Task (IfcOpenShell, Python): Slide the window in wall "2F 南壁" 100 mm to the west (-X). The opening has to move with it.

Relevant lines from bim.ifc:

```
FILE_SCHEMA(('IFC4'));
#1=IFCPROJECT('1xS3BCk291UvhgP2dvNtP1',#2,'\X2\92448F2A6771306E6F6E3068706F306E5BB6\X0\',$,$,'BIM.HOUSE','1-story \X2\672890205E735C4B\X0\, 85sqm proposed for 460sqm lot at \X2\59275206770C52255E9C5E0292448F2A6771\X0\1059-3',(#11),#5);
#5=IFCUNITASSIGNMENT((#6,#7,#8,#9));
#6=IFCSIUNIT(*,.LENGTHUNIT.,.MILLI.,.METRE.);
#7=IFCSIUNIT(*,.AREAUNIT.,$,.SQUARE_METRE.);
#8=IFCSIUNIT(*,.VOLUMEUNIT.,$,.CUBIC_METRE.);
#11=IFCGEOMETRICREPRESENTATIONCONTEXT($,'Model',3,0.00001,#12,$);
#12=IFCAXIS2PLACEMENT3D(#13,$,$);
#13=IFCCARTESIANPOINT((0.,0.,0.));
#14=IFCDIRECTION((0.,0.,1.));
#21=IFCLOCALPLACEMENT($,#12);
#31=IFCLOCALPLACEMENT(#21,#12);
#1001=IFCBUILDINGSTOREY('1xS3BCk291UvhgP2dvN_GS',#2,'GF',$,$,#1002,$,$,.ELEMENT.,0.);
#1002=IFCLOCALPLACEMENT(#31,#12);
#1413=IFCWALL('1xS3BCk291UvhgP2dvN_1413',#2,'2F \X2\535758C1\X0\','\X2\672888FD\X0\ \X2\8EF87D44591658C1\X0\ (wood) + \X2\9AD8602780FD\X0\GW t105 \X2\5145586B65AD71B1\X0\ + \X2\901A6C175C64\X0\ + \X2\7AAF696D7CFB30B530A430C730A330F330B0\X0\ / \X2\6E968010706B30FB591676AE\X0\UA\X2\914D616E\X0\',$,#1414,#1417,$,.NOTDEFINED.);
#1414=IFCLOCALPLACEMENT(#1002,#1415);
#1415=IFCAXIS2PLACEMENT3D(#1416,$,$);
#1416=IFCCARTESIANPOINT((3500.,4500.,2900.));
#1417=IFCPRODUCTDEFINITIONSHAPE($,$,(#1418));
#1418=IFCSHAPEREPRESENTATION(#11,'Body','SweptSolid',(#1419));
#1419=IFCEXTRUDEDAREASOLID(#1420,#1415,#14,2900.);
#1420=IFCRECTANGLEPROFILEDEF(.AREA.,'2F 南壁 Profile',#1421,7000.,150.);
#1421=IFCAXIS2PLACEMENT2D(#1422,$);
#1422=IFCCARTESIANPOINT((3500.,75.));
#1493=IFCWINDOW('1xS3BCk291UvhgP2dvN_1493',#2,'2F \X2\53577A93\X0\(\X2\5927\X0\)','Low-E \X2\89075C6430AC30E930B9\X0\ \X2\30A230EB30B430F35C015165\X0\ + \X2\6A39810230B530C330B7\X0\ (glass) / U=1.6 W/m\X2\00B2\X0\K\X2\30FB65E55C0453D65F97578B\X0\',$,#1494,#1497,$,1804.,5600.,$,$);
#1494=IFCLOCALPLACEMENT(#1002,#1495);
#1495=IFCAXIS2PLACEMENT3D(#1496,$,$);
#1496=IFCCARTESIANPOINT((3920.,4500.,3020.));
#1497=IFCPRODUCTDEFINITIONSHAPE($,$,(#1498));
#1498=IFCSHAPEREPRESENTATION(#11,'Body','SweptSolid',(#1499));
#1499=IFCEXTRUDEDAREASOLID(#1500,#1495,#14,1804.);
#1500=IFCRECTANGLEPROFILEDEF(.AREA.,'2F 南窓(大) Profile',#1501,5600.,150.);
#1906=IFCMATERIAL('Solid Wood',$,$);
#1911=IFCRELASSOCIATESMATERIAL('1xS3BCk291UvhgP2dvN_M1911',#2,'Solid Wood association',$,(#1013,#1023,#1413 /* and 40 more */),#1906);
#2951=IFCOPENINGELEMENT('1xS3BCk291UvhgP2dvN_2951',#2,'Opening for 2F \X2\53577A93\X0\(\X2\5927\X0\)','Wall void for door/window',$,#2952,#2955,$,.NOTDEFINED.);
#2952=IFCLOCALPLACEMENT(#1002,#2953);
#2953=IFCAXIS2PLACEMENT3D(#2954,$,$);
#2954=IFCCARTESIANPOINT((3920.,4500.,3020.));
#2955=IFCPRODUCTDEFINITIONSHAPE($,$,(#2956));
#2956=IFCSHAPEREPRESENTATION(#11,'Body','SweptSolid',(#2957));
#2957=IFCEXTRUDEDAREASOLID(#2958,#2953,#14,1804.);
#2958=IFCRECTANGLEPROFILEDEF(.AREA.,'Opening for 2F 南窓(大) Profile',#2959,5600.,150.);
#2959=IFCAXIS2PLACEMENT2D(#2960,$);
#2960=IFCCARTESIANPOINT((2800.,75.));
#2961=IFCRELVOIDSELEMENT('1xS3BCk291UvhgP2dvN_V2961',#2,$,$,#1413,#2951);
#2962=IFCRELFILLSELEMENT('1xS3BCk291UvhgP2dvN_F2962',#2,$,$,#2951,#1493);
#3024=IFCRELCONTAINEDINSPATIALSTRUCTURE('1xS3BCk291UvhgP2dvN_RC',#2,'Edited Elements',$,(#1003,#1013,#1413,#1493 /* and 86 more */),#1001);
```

```python
import ifcopenshell
import ifcopenshell.api.geometry
import ifcopenshell.util.placement

model = ifcopenshell.open("bim.ifc")

window = model.by_guid("1xS3BCk291UvhgP2dvN_1493")
opening = window.FillsVoids[0].RelatingOpeningElement
wall = opening.VoidsElements[0].RelatingBuildingElement

wall_matrix = ifcopenshell.util.placement.get_local_placement(wall.ObjectPlacement)
shift = wall_matrix[:3, 0] * -100.0
before = ifcopenshell.util.placement.get_local_placement(window.ObjectPlacement)[:3, 3].copy()

# The window is not placed relative to its opening, so move both.
for product in (opening, window):
    matrix = ifcopenshell.util.placement.get_local_placement(product.ObjectPlacement)
    matrix[:3, 3] += shift
    ifcopenshell.api.geometry.edit_object_placement(model, product=product, matrix=matrix, is_si=False)

after = ifcopenshell.util.placement.get_local_placement(window.ObjectPlacement)[:3, 3]
print("window moved by", (after - before).round(3) + 0.0)

model.write("bim_updated.ifc")
```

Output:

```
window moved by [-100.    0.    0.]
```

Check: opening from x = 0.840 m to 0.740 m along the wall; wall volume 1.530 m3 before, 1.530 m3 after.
